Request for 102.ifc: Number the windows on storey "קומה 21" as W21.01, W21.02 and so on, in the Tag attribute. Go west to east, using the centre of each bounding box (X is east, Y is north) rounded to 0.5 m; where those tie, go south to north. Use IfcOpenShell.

First a look at what the model holds.

```python
import ifcopenshell
import ifcopenshell.util.element
import ifcopenshell.util.placement

model = ifcopenshell.open("102.ifc")
print(model.schema)
storey = next(s for s in model.by_type("IfcBuildingStorey") if s.Name == "קומה 21")
windows = [e for e in ifcopenshell.util.element.get_decomposition(storey) if e.is_a("IfcWindow")]
for e in sorted(windows, key=lambda e: e.id()):
    origin = ifcopenshell.util.placement.get_local_placement(e.ObjectPlacement)[:3, 3]
    print(e.id(), e.Tag, e.Name, origin.round(2) + 0.0, sep=" | ")
```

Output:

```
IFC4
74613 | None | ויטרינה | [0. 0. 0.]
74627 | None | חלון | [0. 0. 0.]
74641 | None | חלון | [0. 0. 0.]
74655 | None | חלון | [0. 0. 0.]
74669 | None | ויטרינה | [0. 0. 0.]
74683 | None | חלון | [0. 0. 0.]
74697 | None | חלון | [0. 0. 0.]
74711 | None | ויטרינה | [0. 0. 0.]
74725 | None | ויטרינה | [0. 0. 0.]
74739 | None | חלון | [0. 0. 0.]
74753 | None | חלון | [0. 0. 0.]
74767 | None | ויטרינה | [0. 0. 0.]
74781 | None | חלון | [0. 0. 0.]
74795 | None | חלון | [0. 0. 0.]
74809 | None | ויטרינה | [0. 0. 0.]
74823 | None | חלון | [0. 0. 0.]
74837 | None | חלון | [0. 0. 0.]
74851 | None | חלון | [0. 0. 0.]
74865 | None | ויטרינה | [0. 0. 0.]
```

```python
import ifcopenshell
import ifcopenshell.geom
import ifcopenshell.util.element
import ifcopenshell.util.shape

model = ifcopenshell.open("102.ifc")
settings = ifcopenshell.geom.settings()
settings.set("use-world-coords", True)


def centre(element):
    shape = ifcopenshell.geom.create_shape(settings, element)
    return ifcopenshell.util.shape.get_bbox_centroid(shape.geometry)


storey = next(s for s in model.by_type("IfcBuildingStorey") if s.Name == "קומה 21")
windows = [e for e in ifcopenshell.util.element.get_decomposition(storey) if e.is_a("IfcWindow")]

# Insertion points can sit at a corner or the storey origin, so sort by the geometry (in metres).
centres = {e: centre(e) for e in windows}
windows.sort(key=lambda e: (round(centres[e][0] / 0.5), centres[e][1]))

for i, e in enumerate(windows, start=1):
    number = f"W21.{i:02d}"
    e.Tag = number
    print(e.id(), number)

model.write("102-out.ifc")
```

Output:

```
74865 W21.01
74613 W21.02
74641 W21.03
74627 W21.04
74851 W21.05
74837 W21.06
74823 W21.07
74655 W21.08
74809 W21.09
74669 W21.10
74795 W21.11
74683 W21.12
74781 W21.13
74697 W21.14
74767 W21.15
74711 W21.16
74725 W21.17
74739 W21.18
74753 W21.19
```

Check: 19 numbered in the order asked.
